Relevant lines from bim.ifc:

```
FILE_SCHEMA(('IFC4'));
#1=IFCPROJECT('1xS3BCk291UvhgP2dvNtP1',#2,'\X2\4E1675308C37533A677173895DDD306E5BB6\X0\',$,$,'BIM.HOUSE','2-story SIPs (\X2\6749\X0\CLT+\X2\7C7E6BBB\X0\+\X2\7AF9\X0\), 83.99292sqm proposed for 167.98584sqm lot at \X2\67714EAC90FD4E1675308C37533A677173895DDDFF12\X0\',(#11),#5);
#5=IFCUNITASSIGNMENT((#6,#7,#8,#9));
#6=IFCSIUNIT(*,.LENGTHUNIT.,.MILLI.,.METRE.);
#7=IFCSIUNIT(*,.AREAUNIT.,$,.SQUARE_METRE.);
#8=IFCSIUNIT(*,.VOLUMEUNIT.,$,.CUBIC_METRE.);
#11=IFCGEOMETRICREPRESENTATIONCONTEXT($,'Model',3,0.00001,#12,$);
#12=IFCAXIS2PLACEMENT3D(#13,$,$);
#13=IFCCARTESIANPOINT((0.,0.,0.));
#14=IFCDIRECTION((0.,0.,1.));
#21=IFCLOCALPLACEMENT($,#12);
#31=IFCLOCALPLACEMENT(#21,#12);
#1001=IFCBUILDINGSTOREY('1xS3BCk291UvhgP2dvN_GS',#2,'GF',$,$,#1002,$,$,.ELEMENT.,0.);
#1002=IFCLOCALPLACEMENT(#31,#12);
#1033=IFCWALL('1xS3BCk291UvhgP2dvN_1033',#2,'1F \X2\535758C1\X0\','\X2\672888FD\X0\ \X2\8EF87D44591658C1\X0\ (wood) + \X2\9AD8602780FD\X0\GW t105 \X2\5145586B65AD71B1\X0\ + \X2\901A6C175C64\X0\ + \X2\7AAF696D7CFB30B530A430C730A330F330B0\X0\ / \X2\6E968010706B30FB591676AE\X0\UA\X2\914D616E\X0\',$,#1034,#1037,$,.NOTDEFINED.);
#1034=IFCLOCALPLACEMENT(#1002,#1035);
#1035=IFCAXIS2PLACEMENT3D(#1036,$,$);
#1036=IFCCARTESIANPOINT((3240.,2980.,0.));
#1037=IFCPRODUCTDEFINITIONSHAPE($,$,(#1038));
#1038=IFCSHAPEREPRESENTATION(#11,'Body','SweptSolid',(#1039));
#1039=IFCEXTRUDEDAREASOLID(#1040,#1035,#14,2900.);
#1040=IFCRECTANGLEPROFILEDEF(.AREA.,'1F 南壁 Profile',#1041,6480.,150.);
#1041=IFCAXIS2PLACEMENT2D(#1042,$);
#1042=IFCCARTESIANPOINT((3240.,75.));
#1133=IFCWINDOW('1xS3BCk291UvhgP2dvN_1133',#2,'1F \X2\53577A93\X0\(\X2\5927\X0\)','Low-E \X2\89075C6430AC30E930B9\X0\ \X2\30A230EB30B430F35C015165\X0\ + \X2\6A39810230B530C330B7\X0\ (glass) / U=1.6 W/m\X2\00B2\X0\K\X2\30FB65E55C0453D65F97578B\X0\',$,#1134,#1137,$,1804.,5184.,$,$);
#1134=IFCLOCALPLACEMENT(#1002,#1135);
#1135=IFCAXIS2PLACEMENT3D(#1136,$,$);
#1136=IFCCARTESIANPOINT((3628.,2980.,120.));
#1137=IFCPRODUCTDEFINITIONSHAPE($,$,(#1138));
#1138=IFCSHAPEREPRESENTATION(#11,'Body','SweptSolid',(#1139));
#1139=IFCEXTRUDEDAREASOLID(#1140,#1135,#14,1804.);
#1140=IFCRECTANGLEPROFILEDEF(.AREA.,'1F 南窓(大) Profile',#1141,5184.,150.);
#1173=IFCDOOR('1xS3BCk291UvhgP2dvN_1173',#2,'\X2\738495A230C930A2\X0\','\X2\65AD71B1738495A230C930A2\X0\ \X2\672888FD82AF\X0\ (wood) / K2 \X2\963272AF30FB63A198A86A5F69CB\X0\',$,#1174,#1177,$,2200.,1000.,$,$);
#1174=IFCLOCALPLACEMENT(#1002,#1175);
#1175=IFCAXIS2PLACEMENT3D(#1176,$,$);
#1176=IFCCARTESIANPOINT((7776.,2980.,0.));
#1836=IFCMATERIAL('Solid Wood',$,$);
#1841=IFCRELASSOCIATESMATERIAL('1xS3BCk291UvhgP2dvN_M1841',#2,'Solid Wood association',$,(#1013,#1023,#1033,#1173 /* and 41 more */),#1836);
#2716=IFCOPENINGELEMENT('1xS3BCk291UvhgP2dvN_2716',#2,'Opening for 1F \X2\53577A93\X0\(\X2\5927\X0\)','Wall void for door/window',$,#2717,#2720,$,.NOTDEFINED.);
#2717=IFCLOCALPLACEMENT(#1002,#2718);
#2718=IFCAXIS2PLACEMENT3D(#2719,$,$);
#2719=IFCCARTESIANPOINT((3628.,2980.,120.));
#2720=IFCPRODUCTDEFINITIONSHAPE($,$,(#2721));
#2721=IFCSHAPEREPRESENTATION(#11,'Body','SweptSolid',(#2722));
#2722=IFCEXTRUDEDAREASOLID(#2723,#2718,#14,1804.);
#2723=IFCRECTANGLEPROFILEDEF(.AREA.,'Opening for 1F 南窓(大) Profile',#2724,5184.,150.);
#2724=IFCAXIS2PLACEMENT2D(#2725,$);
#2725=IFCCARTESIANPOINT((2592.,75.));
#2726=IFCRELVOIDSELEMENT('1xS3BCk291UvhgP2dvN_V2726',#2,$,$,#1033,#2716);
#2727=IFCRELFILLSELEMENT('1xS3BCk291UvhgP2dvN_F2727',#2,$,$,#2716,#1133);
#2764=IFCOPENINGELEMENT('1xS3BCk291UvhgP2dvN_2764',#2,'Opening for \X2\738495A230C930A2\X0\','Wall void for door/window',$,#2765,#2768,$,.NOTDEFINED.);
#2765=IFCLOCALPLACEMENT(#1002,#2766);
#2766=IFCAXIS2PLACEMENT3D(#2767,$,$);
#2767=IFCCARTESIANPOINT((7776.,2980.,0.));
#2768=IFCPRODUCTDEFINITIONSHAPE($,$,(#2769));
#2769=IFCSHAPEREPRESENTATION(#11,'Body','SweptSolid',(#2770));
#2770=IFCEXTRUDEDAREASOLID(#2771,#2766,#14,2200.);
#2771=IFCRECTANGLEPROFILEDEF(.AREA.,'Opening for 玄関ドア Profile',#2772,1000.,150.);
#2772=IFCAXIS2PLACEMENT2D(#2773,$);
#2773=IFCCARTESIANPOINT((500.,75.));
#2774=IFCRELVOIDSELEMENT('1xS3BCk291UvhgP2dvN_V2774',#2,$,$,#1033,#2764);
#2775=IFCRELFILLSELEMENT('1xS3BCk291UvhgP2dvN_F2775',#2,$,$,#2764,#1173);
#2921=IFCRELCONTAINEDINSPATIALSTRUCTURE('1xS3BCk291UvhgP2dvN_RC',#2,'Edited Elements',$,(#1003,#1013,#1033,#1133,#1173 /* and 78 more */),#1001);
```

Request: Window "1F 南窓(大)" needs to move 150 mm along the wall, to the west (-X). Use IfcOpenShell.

```python
import ifcopenshell
import ifcopenshell.api.geometry
import ifcopenshell.util.placement
import ifcopenshell.util.unit

model = ifcopenshell.open("bim.ifc")
unit_scale = ifcopenshell.util.unit.calculate_unit_scale(model)

window = model.by_id(1133)
opening = window.FillsVoids[0].RelatingOpeningElement
wall = opening.VoidsElements[0].RelatingBuildingElement

wall_matrix = ifcopenshell.util.placement.get_local_placement(wall.ObjectPlacement)
shift = wall_matrix[:3, 0] * -0.15 / unit_scale
before = ifcopenshell.util.placement.get_local_placement(window.ObjectPlacement)[:3, 3].copy()

# The window is not placed relative to its opening, so move both.
for product in (opening, window):
    matrix = ifcopenshell.util.placement.get_local_placement(product.ObjectPlacement)
    matrix[:3, 3] += shift
    ifcopenshell.api.geometry.edit_object_placement(model, product=product, matrix=matrix, is_si=False)

after = ifcopenshell.util.placement.get_local_placement(window.ObjectPlacement)[:3, 3]
print("window moved by", (after - before).round(3) + 0.0)

model.write("bim_edited.ifc")
```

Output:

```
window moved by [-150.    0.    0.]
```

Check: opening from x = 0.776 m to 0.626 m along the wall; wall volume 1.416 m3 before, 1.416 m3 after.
